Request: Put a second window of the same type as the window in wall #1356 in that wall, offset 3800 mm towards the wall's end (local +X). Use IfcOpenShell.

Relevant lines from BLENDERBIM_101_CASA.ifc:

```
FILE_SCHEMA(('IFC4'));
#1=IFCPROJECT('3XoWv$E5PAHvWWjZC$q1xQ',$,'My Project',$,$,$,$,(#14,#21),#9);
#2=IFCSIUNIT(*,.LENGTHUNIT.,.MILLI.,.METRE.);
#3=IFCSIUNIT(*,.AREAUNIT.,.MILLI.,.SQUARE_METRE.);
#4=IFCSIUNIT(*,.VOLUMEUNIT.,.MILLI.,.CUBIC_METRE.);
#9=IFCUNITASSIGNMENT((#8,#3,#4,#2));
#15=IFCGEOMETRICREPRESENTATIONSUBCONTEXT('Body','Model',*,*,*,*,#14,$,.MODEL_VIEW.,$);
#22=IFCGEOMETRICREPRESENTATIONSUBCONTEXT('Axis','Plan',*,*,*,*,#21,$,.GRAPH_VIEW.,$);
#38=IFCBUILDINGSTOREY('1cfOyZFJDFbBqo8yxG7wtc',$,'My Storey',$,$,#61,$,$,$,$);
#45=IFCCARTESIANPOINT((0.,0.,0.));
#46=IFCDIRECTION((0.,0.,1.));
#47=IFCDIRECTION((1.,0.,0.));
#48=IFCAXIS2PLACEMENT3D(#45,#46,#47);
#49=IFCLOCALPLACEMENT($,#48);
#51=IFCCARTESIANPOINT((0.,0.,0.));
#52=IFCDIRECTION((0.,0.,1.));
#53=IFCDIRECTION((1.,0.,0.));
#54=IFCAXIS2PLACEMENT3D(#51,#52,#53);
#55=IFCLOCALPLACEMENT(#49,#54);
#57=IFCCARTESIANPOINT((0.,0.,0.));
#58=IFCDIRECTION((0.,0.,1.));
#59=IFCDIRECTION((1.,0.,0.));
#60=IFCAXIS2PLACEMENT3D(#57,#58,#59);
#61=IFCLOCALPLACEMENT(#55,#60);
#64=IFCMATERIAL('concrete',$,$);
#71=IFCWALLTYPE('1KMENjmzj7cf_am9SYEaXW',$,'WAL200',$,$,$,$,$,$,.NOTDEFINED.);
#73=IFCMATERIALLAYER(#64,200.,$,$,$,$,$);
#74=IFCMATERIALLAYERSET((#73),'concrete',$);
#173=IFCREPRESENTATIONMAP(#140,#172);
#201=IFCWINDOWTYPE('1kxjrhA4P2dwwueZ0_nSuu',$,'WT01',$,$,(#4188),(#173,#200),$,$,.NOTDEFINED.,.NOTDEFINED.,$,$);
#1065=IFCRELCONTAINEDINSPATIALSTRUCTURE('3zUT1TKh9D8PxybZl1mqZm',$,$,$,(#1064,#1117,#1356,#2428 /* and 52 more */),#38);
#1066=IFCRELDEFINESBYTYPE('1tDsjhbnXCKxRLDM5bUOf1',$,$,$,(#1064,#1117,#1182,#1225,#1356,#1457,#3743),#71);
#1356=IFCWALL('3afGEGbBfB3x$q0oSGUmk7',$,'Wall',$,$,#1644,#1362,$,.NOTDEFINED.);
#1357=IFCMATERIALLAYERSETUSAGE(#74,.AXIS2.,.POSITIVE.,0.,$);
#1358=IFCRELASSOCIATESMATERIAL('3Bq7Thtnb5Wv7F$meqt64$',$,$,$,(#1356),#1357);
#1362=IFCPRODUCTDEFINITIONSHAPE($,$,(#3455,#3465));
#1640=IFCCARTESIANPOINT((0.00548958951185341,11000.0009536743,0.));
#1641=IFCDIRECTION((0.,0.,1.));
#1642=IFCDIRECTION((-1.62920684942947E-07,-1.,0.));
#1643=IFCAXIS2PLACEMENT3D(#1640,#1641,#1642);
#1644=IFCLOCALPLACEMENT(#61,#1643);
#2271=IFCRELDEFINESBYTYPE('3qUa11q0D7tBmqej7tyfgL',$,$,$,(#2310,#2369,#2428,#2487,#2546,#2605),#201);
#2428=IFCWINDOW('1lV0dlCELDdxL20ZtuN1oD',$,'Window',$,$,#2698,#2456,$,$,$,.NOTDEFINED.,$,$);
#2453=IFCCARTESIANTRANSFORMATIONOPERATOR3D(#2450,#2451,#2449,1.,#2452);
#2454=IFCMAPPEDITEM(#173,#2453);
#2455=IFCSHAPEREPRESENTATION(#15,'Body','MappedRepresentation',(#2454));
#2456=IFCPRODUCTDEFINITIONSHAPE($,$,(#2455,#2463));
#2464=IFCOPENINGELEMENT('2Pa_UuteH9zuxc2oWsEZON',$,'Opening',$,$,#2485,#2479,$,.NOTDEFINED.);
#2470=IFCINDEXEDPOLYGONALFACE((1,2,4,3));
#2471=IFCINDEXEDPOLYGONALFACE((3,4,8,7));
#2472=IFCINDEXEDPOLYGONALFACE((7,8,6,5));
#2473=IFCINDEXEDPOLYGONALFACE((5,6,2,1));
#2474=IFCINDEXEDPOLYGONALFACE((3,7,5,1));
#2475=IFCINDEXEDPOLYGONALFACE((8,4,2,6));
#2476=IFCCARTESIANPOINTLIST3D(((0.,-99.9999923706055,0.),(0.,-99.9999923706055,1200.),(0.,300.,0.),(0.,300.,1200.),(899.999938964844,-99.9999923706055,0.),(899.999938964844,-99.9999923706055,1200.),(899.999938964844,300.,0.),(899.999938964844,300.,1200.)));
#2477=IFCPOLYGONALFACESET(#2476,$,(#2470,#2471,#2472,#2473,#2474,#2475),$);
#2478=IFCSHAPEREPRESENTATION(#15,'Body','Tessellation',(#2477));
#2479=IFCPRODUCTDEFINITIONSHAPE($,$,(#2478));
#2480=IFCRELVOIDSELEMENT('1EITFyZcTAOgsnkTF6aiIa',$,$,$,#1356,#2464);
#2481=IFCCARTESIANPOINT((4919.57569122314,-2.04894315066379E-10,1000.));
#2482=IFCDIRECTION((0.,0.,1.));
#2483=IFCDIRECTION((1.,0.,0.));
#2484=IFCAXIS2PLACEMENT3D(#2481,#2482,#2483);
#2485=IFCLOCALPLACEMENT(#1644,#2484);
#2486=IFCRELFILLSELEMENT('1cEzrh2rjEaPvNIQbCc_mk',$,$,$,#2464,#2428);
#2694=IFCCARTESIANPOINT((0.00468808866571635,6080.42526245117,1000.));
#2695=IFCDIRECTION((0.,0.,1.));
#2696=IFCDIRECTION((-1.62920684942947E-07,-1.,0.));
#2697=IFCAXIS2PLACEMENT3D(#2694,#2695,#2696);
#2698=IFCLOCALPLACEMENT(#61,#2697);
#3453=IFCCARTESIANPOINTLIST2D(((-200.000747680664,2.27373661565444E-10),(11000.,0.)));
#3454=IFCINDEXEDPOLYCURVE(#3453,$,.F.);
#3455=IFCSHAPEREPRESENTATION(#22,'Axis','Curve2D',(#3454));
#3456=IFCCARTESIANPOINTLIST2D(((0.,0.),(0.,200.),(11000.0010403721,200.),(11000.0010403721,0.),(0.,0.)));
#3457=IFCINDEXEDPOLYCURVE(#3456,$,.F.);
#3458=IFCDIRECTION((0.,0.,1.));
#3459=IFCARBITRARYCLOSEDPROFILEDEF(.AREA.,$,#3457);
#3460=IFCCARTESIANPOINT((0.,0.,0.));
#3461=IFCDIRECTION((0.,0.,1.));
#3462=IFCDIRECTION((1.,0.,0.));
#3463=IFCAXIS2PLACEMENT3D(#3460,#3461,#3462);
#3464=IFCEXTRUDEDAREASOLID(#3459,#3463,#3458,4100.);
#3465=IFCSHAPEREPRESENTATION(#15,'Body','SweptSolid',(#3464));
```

```python
import ifcopenshell
import ifcopenshell.api.feature
import ifcopenshell.api.geometry
import ifcopenshell.api.root
import ifcopenshell.geom
import ifcopenshell.util.element
import ifcopenshell.util.placement
import ifcopenshell.util.shape

model = ifcopenshell.open("BLENDERBIM_101_CASA.ifc")
settings = ifcopenshell.geom.settings()


def volume(element):
    """Net volume in cubic metres, openings subtracted."""
    shape = ifcopenshell.geom.create_shape(settings, element)
    return ifcopenshell.util.shape.get_volume(shape.geometry)


window = model.by_guid("1lV0dlCELDdxL20ZtuN1oD")
opening = window.FillsVoids[0].RelatingOpeningElement
wall = opening.VoidsElements[0].RelatingBuildingElement
before = volume(wall)
shift = ifcopenshell.util.placement.get_local_placement(wall.ObjectPlacement)[:3, 0] * 3800.0

# copy_class copies the void relationship, type, container and properties, but no geometry.
new_opening = ifcopenshell.api.root.copy_class(model, product=opening)
new_opening.Representation = ifcopenshell.util.element.copy_deep(
    model, opening.Representation, exclude=["IfcGeometricRepresentationContext", "IfcRepresentationMap"]
)
new_window = ifcopenshell.api.root.copy_class(model, product=window)
new_window.Representation = ifcopenshell.util.element.copy_deep(
    model, window.Representation, exclude=["IfcGeometricRepresentationContext", "IfcRepresentationMap"]
)
ifcopenshell.api.feature.add_filling(model, opening=new_opening, element=new_window)

for old, new in ((opening, new_opening), (window, new_window)):
    matrix = ifcopenshell.util.placement.get_local_placement(old.ObjectPlacement)
    matrix[:3, 3] += shift
    ifcopenshell.api.geometry.edit_object_placement(model, product=new, matrix=matrix, is_si=False)

after = volume(wall)

print(f"wall volume {before:.3f} -> {after:.3f} m3")

model.write("BLENDERBIM_101_CASA_rev.ifc")
```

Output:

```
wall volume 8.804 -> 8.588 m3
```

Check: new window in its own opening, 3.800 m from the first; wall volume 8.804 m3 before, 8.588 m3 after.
